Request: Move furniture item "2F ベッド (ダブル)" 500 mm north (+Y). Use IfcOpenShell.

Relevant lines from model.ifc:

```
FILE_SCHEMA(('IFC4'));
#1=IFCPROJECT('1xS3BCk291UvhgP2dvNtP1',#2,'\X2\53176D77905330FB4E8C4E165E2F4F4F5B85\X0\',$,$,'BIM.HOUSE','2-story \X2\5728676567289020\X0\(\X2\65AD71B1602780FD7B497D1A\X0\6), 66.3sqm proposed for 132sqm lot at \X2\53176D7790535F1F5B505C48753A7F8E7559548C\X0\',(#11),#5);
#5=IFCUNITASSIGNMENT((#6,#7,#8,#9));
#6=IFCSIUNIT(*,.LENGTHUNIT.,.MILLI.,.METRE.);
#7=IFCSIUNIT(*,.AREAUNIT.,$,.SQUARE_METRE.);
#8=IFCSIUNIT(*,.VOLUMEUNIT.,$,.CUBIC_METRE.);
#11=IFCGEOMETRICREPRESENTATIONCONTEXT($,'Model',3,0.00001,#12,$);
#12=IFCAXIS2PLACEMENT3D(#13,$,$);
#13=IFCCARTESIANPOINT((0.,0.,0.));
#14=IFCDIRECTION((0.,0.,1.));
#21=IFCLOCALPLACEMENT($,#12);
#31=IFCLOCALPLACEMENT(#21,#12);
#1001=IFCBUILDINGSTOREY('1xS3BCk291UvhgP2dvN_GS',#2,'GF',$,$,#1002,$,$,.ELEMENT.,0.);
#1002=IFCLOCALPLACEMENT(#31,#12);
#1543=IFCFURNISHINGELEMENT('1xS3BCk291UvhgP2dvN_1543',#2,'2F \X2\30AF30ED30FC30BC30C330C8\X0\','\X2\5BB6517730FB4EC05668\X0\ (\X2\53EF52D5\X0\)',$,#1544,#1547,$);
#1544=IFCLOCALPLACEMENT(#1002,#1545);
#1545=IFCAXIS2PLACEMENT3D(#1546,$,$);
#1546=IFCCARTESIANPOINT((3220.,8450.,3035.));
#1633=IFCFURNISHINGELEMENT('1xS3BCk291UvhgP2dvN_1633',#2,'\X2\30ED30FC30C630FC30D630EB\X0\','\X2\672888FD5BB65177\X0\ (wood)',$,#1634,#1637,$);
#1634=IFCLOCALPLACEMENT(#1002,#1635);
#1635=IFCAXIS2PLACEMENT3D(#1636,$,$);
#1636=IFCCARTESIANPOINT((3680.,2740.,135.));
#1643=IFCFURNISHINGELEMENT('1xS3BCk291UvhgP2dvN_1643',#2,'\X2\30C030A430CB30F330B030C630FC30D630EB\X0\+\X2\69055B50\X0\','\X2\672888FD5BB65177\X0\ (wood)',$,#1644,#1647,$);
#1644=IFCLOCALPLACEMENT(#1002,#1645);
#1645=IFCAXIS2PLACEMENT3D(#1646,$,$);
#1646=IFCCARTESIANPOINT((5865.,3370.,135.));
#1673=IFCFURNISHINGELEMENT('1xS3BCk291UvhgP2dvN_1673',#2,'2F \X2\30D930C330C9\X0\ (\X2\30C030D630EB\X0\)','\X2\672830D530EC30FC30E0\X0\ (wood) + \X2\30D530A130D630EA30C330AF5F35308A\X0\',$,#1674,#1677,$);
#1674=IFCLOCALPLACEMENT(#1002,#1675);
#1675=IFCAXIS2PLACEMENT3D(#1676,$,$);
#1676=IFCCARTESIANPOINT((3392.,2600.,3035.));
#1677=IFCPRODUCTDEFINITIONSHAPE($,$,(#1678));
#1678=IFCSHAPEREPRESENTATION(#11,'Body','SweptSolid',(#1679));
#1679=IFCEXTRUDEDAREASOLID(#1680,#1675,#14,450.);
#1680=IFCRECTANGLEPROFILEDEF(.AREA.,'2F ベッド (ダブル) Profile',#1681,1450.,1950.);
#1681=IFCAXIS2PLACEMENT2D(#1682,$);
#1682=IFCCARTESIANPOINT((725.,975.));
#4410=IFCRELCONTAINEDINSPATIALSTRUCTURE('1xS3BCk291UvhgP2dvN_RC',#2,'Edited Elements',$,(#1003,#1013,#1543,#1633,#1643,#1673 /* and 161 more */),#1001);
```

```python
import ifcopenshell
import ifcopenshell.api.geometry
import ifcopenshell.util.placement
import ifcopenshell.util.unit

model = ifcopenshell.open("model.ifc")
unit_scale = ifcopenshell.util.unit.calculate_unit_scale(model)

item = model.by_id(1673)
matrix = ifcopenshell.util.placement.get_local_placement(item.ObjectPlacement)
matrix[1, 3] += 0.5 / unit_scale
ifcopenshell.api.geometry.edit_object_placement(model, product=item, matrix=matrix, is_si=False)

print(ifcopenshell.util.placement.get_local_placement(item.ObjectPlacement).round(3) + 0.0)

model.write("model_edited.ifc")
```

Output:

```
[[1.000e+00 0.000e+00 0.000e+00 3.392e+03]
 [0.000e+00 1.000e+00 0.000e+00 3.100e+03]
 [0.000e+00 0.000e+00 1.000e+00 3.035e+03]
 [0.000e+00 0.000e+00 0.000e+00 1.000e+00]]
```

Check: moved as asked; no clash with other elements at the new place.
